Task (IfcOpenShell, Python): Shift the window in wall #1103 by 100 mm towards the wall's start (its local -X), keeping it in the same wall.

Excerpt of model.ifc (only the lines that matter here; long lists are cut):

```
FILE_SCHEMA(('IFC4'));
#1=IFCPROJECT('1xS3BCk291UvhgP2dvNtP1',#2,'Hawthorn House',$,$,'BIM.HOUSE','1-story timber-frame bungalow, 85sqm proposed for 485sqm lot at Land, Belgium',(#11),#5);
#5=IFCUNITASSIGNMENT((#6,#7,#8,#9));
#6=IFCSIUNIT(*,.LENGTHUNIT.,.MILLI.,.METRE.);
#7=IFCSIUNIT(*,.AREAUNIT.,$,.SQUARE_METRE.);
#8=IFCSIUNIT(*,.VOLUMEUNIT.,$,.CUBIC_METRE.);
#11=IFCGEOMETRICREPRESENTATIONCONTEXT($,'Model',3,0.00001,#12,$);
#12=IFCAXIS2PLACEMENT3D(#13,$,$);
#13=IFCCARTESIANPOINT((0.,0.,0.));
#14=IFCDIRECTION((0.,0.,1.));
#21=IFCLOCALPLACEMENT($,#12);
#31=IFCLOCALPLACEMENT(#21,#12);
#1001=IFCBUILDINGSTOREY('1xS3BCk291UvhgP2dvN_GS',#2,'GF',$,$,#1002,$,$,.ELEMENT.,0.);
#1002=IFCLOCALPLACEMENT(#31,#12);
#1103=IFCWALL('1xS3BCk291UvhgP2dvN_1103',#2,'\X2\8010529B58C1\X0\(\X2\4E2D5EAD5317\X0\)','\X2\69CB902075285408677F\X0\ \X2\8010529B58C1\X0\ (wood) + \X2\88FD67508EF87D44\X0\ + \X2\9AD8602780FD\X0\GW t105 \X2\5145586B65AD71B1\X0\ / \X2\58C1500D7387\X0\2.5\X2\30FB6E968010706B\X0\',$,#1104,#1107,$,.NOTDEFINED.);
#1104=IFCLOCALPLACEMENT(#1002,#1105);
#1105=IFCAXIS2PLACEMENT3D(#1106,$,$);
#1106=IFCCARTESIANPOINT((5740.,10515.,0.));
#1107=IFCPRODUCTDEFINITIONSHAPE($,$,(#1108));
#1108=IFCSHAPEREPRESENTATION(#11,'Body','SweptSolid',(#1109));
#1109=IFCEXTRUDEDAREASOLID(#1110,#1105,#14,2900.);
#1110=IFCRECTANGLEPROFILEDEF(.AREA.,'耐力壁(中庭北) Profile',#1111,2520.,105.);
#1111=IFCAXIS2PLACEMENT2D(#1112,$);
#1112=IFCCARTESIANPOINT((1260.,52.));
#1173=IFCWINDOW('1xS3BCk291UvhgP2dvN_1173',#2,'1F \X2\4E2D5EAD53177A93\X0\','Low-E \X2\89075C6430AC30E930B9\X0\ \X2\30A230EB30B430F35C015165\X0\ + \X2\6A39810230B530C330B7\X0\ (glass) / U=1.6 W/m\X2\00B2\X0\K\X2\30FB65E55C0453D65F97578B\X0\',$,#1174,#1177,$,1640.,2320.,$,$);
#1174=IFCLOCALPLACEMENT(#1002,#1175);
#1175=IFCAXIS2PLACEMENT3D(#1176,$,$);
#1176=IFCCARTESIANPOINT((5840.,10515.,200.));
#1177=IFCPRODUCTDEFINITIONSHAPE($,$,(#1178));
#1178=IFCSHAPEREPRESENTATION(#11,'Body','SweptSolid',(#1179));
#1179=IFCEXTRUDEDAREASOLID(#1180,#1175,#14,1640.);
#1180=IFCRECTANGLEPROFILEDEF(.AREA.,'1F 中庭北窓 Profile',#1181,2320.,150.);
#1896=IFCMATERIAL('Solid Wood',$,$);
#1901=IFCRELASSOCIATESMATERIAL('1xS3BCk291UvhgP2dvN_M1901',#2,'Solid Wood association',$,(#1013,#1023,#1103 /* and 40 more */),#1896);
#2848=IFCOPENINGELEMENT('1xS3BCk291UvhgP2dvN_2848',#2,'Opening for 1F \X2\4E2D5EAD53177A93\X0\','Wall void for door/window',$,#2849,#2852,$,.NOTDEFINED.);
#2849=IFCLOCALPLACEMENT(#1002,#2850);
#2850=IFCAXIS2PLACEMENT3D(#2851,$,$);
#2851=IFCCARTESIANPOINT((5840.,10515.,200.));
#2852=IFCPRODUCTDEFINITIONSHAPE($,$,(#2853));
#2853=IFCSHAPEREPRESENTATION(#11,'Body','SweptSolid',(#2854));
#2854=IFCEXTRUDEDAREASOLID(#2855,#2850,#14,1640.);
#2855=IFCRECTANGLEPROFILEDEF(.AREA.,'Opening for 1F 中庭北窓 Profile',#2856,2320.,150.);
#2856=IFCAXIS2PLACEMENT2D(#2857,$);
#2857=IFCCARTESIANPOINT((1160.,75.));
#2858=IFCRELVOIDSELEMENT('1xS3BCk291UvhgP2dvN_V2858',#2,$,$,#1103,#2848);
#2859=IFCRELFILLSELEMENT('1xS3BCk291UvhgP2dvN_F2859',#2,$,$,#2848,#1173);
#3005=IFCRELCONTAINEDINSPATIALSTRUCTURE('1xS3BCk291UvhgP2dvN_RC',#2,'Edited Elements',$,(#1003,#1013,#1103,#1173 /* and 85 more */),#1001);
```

```python
import ifcopenshell
import ifcopenshell.api.geometry
import ifcopenshell.util.placement
import ifcopenshell.util.unit

model = ifcopenshell.open("model.ifc")
unit_scale = ifcopenshell.util.unit.calculate_unit_scale(model)

window = model.by_guid("1xS3BCk291UvhgP2dvN_1173")
opening = window.FillsVoids[0].RelatingOpeningElement
wall = opening.VoidsElements[0].RelatingBuildingElement

wall_matrix = ifcopenshell.util.placement.get_local_placement(wall.ObjectPlacement)
shift = wall_matrix[:3, 0] * -0.1 / unit_scale
before = ifcopenshell.util.placement.get_local_placement(window.ObjectPlacement)[:3, 3].copy()

# The window is not placed relative to its opening, so move both.
for product in (opening, window):
    matrix = ifcopenshell.util.placement.get_local_placement(product.ObjectPlacement)
    matrix[:3, 3] += shift
    ifcopenshell.api.geometry.edit_object_placement(model, product=product, matrix=matrix, is_si=False)

after = ifcopenshell.util.placement.get_local_placement(window.ObjectPlacement)[:3, 3]
print("window moved by", (after - before).round(3) + 0.0)

model.write("model_v2.ifc")
```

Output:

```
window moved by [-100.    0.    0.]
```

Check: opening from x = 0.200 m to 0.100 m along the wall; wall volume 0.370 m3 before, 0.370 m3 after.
